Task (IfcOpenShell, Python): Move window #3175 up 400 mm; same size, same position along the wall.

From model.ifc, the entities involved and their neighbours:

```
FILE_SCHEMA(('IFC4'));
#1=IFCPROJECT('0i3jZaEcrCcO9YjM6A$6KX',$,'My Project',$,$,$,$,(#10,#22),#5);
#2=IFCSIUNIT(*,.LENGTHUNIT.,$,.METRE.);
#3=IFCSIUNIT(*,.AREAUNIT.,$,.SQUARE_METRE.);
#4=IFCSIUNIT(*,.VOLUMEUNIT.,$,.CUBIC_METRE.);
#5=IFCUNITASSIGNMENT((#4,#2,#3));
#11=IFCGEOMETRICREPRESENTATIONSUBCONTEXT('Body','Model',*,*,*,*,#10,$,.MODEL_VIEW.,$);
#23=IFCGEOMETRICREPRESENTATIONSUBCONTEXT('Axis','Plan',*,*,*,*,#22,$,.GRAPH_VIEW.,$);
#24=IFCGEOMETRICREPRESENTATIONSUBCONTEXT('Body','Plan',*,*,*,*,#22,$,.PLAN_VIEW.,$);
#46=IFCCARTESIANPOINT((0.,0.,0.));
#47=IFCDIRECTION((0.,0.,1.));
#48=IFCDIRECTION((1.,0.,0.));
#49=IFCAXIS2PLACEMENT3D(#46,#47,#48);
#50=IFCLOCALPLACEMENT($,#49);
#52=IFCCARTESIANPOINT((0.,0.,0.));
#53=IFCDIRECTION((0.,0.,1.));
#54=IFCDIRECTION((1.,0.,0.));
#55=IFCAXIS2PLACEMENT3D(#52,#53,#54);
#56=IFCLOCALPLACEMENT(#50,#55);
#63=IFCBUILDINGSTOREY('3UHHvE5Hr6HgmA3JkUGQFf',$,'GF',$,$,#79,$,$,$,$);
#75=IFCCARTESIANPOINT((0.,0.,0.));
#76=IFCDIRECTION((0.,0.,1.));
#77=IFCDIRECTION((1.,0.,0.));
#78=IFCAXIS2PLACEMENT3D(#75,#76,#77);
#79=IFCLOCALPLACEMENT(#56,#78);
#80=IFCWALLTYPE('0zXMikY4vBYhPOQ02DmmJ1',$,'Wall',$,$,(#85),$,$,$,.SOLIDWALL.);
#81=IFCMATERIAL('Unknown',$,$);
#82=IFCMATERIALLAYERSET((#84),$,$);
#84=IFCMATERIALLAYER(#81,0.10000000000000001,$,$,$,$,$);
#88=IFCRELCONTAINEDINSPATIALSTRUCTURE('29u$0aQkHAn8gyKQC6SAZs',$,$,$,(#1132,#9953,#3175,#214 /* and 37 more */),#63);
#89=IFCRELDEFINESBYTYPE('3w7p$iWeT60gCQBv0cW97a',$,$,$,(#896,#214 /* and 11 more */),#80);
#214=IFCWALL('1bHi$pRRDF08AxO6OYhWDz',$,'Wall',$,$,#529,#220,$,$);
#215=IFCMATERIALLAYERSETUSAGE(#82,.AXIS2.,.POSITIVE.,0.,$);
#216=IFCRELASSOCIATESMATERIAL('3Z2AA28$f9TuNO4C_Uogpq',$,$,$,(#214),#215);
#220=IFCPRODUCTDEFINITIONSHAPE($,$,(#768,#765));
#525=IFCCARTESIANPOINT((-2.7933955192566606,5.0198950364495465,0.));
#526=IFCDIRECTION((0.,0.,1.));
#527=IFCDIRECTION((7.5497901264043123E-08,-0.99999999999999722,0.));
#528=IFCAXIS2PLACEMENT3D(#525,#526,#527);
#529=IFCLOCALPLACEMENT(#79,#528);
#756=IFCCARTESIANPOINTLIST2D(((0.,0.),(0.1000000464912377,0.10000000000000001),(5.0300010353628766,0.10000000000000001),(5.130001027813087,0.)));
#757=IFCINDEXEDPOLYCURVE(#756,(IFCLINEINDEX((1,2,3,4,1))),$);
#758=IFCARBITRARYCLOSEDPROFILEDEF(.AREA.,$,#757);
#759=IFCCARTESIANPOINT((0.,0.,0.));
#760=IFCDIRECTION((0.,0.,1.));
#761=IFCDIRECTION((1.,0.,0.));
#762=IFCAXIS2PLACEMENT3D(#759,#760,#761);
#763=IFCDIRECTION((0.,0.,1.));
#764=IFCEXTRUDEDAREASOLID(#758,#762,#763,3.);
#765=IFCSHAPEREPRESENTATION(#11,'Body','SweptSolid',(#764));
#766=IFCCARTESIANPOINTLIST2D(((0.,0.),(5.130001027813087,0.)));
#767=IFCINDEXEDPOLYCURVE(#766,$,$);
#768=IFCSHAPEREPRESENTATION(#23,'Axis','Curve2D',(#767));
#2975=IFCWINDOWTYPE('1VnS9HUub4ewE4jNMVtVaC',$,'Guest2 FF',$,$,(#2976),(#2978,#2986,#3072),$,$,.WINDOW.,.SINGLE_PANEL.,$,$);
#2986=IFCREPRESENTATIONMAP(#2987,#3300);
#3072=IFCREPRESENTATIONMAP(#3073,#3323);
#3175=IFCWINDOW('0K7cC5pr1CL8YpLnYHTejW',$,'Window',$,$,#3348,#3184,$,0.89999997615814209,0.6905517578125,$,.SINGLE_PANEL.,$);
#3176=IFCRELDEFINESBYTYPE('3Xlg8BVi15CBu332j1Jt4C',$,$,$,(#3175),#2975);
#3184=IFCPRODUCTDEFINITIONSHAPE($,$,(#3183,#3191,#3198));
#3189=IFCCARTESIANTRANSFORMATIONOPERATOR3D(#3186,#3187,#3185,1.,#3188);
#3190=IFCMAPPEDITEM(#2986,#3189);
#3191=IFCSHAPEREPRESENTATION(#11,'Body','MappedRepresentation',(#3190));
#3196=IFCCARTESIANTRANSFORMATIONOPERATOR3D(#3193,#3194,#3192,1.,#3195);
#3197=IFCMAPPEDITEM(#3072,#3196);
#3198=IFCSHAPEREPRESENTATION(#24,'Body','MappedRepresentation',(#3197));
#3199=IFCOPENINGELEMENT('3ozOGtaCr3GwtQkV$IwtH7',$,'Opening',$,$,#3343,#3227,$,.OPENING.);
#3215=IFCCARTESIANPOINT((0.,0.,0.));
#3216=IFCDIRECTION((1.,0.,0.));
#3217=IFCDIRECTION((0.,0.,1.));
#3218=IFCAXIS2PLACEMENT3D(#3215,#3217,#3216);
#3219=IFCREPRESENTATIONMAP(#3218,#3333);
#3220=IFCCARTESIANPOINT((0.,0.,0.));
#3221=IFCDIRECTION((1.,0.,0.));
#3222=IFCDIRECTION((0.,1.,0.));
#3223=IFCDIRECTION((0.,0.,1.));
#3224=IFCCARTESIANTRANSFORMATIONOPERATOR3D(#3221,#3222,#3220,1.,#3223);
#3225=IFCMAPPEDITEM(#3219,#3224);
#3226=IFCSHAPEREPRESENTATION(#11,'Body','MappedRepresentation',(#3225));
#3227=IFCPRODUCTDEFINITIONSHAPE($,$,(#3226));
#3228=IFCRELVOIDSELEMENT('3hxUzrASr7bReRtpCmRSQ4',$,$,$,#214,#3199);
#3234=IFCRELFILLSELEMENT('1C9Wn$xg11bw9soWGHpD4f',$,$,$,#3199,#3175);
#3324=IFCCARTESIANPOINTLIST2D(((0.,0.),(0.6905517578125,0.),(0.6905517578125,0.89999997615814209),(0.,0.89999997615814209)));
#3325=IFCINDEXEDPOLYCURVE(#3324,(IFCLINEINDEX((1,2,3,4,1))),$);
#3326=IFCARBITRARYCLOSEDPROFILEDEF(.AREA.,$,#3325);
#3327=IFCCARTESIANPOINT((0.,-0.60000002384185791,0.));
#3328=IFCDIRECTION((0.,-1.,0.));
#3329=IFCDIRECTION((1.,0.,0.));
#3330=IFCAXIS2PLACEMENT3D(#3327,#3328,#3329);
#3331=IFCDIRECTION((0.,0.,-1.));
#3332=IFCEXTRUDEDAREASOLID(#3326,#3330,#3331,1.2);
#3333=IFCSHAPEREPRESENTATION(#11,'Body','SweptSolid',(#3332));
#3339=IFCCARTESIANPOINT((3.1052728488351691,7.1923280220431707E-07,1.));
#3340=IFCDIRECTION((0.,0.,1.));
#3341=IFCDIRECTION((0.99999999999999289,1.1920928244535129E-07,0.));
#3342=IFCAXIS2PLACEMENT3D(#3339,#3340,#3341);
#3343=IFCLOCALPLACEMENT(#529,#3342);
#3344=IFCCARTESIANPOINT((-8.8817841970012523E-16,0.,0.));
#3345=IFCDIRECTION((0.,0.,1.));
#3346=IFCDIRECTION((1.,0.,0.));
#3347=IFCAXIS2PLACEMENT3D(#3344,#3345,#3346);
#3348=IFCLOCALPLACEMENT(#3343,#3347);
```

```python
import numpy as np
import ifcopenshell
import ifcopenshell.api.geometry
import ifcopenshell.util.placement
import ifcopenshell.util.unit

model = ifcopenshell.open("model.ifc")
unit_scale = ifcopenshell.util.unit.calculate_unit_scale(model)

window = model.by_guid("0K7cC5pr1CL8YpLnYHTejW")
opening = window.FillsVoids[0].RelatingOpeningElement
dz = 0.4

shift = np.array([0.0, 0.0, dz])
# The window is placed relative to its opening, so it follows when the opening moves.
matrix = ifcopenshell.util.placement.get_local_placement(opening.ObjectPlacement)
matrix[:3, 3] += shift
ifcopenshell.api.geometry.edit_object_placement(
    model, product=opening, matrix=matrix, is_si=False, should_transform_children=True
)

print(f"moved by {dz * unit_scale:+.3f} m")

model.write("model-out.ifc")
```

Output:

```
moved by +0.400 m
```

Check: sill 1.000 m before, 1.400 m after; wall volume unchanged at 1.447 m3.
